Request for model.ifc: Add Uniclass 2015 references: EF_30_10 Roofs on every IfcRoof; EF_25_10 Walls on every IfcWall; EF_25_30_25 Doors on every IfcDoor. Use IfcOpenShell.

First a look at what the model holds.

```python
import ifcopenshell

model = ifcopenshell.open("model.ifc")
print(model.schema)
print("classifications:", [c.Name for c in model.by_type("IfcClassification")])
for ifc_class in ("IfcDoor", "IfcRoof", "IfcStair", "IfcWall", "IfcWindow"):
    print(ifc_class, len(model.by_type(ifc_class)))
```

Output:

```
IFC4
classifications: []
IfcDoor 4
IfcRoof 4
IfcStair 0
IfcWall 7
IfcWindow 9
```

```python
import ifcopenshell
import ifcopenshell.api.classification

model = ifcopenshell.open("model.ifc")

system = ifcopenshell.api.classification.add_classification(model, classification="Uniclass 2015")

codes = {
    "IfcRoof": ("EF_30_10", "Roofs"),
    "IfcWall": ("EF_25_10", "Walls"),
    "IfcDoor": ("EF_25_30_25", "Doors"),
}
for ifc_class, (code, name) in codes.items():
    products = model.by_type(ifc_class)
    ifcopenshell.api.classification.add_reference(
        model, products=products, classification=system, identification=code, name=name
    )
    print(code, len(products))

model.write("model_updated.ifc")
```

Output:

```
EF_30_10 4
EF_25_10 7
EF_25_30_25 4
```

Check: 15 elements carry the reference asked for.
